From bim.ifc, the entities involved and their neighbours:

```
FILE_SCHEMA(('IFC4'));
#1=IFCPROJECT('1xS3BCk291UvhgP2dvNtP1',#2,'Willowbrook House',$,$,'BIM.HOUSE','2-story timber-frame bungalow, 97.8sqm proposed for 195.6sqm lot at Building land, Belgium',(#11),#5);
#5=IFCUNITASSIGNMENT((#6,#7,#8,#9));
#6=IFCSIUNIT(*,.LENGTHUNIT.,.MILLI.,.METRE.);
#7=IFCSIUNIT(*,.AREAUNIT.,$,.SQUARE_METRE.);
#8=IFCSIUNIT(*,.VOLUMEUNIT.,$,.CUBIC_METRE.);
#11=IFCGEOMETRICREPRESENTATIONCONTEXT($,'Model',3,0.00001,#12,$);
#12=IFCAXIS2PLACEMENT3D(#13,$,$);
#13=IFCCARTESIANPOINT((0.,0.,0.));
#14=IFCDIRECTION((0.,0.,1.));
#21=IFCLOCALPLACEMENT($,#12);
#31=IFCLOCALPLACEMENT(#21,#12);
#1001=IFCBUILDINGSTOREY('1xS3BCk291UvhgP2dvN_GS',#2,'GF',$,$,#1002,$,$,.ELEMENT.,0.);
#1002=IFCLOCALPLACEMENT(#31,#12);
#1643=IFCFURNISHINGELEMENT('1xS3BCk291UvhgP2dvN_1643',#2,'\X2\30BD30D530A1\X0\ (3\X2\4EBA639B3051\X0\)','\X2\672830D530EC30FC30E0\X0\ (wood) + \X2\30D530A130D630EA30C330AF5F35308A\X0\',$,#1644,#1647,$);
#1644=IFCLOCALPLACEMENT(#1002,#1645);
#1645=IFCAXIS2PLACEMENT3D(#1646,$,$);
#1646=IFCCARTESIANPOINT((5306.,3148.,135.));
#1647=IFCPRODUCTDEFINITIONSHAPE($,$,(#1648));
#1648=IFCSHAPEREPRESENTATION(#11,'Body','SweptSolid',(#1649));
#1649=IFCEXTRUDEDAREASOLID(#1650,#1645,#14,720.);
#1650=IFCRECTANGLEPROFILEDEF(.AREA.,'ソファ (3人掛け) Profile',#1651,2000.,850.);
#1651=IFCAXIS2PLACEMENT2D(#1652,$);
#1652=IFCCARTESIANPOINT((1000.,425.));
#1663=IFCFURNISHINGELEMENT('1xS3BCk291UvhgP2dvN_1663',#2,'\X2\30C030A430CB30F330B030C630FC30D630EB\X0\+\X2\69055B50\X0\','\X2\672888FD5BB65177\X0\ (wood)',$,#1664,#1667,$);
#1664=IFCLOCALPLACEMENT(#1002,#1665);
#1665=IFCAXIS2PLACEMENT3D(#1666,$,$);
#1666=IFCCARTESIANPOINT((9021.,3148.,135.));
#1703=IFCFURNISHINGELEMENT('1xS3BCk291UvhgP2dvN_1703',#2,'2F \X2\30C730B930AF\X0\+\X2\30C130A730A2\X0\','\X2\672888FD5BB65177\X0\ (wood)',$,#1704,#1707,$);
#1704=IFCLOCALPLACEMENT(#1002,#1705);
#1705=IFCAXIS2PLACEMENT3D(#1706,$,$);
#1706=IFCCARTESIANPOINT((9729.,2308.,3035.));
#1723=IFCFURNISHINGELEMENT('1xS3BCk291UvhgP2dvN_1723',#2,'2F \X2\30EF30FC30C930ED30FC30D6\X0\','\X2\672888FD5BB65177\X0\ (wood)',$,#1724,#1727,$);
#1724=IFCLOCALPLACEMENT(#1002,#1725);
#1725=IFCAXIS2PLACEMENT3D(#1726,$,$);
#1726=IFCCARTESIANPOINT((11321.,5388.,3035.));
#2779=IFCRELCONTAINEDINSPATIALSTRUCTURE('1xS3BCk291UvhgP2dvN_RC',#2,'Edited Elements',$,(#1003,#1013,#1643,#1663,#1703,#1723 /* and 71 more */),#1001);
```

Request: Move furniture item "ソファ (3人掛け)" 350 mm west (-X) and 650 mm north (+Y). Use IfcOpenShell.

```python
import ifcopenshell
import ifcopenshell.api.geometry
import ifcopenshell.util.placement

model = ifcopenshell.open("bim.ifc")

item = model.by_guid("1xS3BCk291UvhgP2dvN_1643")
matrix = ifcopenshell.util.placement.get_local_placement(item.ObjectPlacement)
matrix[0, 3] -= 350.0
matrix[1, 3] += 650.0
ifcopenshell.api.geometry.edit_object_placement(model, product=item, matrix=matrix, is_si=False)

print(ifcopenshell.util.placement.get_local_placement(item.ObjectPlacement).round(3) + 0.0)

model.write("bim_rev.ifc")
```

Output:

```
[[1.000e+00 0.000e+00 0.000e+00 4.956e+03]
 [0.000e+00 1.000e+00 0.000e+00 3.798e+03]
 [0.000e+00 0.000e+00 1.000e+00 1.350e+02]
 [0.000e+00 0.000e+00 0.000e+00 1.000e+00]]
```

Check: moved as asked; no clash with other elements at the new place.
